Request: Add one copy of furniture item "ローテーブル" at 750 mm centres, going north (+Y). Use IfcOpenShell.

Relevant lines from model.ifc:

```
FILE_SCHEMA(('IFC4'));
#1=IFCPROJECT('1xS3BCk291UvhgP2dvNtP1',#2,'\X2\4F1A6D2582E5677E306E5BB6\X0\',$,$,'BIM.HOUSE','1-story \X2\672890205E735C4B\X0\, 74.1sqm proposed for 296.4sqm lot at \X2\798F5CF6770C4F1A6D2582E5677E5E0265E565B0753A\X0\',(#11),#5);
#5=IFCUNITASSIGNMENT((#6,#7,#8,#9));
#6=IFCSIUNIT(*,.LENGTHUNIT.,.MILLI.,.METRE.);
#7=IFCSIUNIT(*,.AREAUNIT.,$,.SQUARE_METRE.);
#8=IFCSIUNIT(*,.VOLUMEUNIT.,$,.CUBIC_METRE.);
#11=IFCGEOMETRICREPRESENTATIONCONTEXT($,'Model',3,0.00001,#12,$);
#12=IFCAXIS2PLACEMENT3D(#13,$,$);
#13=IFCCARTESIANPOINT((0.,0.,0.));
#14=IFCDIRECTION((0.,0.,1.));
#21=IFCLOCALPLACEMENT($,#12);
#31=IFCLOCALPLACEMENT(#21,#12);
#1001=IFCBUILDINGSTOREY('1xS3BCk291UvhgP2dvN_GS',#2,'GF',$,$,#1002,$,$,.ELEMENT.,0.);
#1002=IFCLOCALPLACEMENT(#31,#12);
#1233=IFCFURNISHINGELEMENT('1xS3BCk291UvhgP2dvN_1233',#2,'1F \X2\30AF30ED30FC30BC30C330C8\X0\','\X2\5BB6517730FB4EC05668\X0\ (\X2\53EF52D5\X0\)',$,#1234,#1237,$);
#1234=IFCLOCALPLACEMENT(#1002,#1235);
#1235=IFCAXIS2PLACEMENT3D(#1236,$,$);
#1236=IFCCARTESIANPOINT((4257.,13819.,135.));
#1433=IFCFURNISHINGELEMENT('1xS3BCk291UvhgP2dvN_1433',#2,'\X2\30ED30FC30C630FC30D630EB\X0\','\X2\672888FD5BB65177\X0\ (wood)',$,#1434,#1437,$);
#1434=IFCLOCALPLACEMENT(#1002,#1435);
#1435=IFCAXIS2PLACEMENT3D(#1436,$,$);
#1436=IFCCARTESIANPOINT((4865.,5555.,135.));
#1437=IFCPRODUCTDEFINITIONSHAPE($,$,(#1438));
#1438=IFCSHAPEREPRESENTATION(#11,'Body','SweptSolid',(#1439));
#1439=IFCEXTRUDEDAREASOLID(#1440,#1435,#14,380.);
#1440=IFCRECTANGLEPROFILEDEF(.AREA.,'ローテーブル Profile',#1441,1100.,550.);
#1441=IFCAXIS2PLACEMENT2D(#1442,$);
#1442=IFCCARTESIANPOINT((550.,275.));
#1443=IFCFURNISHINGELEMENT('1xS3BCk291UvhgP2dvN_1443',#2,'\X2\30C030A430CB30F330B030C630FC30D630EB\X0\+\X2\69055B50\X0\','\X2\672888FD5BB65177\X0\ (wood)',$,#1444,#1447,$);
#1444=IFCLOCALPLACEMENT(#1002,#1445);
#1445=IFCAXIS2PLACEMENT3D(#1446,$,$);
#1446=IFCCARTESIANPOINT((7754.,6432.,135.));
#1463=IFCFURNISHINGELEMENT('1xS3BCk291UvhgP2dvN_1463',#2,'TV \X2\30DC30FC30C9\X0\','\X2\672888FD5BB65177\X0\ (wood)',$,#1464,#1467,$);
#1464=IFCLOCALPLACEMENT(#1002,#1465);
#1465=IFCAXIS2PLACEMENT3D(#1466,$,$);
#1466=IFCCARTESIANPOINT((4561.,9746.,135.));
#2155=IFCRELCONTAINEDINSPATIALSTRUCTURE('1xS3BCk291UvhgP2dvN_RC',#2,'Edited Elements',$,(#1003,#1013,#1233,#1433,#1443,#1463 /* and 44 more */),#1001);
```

```python
import numpy as np
import ifcopenshell
import ifcopenshell.api.geometry
import ifcopenshell.api.root
import ifcopenshell.util.element
import ifcopenshell.util.placement

model = ifcopenshell.open("model.ifc")


def reuse_history(source, copy):
    """copy_class also copies each property set's owner history, people and application; keep the originals."""
    for rel in copy.IsDefinedBy:
        if rel.is_a("IfcRelDefinesByProperties") and (history := rel.RelatingPropertyDefinition.OwnerHistory):
            rel.RelatingPropertyDefinition.OwnerHistory = source.OwnerHistory
            ifcopenshell.util.element.remove_deep2(model, history)


source = model.by_id(1433)
base = ifcopenshell.util.placement.get_local_placement(source.ObjectPlacement)
step = np.array([0.0, 1.0, 0.0]) * 750.0

for i in range(1, 2):
    copy = ifcopenshell.api.root.copy_class(model, product=source)
    copy.Representation = ifcopenshell.util.element.copy_deep(
        model, source.Representation, exclude=["IfcGeometricRepresentationContext", "IfcRepresentationMap"]
    )
    reuse_history(source, copy)
    matrix = base.copy()
    matrix[:3, 3] += i * step
    print("added at", matrix[:3, 3].round(3) + 0.0)
    ifcopenshell.api.geometry.edit_object_placement(model, product=copy, matrix=matrix, is_si=False)

model.write("model-out.ifc")
```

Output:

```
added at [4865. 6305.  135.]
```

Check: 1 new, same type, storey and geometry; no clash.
